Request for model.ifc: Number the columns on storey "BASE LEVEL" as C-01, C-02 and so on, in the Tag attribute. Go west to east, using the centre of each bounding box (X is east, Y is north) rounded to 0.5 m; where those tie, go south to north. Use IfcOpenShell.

First a look at what the model holds.

```python
import ifcopenshell
import ifcopenshell.util.element
import ifcopenshell.util.placement

model = ifcopenshell.open("model.ifc")
print(model.schema)
storey = next(s for s in model.by_type("IfcBuildingStorey") if s.Name == "BASE LEVEL")
columns = [e for e in ifcopenshell.util.element.get_decomposition(storey) if e.is_a("IfcColumn")]
for e in sorted(columns, key=lambda e: e.id()):
    origin = ifcopenshell.util.placement.get_local_placement(e.ObjectPlacement)[:3, 3]
    print(e.id(), e.Tag, e.Name, origin.round(2) + 0.0, sep=" | ")
```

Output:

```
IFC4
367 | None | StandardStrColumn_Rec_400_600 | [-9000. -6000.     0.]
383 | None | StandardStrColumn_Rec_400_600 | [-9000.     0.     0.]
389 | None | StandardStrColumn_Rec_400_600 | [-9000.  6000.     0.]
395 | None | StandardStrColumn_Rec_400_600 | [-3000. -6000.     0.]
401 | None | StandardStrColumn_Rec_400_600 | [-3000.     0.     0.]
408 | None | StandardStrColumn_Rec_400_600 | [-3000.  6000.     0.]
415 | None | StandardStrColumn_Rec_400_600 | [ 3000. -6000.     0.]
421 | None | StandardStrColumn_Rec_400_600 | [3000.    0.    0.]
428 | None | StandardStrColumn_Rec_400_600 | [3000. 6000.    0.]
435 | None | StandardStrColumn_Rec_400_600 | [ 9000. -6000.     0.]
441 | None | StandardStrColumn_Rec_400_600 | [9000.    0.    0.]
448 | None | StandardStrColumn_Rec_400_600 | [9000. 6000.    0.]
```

```python
import ifcopenshell
import ifcopenshell.geom
import ifcopenshell.util.element
import ifcopenshell.util.shape

model = ifcopenshell.open("model.ifc")
settings = ifcopenshell.geom.settings()
settings.set("use-world-coords", True)


def centre(element):
    shape = ifcopenshell.geom.create_shape(settings, element)
    return ifcopenshell.util.shape.get_bbox_centroid(shape.geometry)


storey = next(s for s in model.by_type("IfcBuildingStorey") if s.Name == "BASE LEVEL")
columns = [e for e in ifcopenshell.util.element.get_decomposition(storey) if e.is_a("IfcColumn")]

# Insertion points can sit at a corner or the storey origin, so sort by the geometry (in metres).
centres = {e: centre(e) for e in columns}
columns.sort(key=lambda e: (round(centres[e][0] / 0.5), centres[e][1]))

for i, e in enumerate(columns, start=1):
    number = f"C-{i:02d}"
    e.Tag = number
    print(e.id(), number)

model.write("model_edited.ifc")
```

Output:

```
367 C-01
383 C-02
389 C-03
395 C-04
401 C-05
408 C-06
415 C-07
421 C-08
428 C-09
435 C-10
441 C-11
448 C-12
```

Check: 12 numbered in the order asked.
